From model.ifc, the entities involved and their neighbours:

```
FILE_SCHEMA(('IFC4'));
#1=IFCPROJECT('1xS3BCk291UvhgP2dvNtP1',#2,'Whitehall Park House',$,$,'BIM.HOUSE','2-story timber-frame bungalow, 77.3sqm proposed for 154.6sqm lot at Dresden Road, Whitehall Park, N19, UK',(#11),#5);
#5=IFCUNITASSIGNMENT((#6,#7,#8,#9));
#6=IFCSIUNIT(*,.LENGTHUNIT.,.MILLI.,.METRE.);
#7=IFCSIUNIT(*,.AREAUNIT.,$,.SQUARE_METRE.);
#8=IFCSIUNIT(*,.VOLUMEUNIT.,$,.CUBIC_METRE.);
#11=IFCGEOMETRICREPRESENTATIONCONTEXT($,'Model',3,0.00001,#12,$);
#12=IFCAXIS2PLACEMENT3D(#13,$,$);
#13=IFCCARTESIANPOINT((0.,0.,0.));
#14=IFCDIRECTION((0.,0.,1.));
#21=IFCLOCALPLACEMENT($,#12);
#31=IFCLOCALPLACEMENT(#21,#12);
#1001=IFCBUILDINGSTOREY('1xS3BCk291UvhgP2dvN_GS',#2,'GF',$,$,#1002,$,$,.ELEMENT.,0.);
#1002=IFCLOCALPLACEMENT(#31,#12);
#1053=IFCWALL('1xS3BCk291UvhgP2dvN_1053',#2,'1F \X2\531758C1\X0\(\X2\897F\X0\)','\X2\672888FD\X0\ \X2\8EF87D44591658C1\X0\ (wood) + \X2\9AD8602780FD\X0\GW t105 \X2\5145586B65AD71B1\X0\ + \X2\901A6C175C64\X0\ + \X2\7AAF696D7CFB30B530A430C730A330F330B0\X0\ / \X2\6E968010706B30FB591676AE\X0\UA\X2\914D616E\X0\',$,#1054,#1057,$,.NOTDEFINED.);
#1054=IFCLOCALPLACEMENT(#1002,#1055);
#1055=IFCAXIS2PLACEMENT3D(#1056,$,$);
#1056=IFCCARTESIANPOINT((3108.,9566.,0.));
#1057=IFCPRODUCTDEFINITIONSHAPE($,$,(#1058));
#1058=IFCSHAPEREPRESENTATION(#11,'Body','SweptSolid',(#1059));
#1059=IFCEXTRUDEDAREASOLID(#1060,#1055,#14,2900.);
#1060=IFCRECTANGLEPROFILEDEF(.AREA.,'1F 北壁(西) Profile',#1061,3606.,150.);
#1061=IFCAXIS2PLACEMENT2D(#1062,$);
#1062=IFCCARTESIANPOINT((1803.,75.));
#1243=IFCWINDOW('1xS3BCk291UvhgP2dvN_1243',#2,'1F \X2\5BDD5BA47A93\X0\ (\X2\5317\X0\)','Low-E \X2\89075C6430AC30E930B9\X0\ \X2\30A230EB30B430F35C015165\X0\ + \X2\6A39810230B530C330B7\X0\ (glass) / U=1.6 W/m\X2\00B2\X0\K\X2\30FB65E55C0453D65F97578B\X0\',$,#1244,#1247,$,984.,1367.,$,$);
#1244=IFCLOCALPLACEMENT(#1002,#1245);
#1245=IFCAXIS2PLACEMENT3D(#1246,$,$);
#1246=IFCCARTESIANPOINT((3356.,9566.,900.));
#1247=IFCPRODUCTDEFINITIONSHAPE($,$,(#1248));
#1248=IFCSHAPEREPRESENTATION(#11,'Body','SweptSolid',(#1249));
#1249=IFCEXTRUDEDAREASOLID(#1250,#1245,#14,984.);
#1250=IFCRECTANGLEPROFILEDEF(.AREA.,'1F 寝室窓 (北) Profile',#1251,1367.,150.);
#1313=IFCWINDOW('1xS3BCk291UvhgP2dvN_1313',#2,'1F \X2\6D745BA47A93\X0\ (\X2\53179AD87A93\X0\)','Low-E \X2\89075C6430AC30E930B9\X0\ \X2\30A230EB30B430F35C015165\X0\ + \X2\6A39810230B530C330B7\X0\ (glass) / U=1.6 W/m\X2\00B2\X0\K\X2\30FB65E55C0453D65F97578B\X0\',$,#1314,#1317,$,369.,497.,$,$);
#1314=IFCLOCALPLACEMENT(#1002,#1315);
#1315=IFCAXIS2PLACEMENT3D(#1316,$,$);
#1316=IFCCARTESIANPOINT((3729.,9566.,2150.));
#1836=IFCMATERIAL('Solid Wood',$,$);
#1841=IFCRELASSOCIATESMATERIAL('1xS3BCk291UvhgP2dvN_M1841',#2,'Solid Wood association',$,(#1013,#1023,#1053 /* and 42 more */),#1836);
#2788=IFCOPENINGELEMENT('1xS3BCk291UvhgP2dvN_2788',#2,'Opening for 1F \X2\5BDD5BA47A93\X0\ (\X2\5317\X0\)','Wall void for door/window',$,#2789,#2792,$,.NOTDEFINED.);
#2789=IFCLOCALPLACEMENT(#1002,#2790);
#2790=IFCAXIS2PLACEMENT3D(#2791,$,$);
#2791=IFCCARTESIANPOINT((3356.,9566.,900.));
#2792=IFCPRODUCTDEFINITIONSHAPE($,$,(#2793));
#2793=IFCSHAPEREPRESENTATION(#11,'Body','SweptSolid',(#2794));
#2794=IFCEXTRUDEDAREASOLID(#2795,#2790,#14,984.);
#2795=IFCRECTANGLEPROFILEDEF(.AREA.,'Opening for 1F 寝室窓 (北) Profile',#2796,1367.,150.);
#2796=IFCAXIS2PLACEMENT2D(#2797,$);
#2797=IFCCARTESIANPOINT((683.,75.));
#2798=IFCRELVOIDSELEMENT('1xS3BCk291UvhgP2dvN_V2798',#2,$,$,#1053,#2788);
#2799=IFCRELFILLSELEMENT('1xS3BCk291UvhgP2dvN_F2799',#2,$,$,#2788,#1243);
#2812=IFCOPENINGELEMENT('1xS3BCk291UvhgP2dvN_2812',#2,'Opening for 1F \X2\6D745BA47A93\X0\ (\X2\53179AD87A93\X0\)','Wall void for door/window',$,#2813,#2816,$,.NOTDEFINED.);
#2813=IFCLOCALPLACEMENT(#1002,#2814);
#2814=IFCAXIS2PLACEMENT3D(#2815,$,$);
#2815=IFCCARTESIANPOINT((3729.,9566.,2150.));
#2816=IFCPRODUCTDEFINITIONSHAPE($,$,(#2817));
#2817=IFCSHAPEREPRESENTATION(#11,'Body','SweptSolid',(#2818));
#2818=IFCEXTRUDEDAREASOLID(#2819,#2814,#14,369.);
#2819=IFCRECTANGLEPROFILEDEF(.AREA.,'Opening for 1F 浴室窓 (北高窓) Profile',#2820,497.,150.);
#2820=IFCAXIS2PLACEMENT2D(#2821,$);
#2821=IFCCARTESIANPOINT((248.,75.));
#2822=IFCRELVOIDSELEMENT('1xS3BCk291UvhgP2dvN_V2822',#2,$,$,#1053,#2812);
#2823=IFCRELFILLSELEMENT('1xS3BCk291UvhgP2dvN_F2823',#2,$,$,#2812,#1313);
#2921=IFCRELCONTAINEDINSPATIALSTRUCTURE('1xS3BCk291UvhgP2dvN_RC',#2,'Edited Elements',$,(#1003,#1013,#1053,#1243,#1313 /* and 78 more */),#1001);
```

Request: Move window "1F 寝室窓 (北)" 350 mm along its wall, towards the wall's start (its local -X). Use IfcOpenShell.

```python
import ifcopenshell
import ifcopenshell.api.geometry
import ifcopenshell.util.placement

model = ifcopenshell.open("model.ifc")

window = model.by_guid("1xS3BCk291UvhgP2dvN_1243")
opening = window.FillsVoids[0].RelatingOpeningElement
wall = opening.VoidsElements[0].RelatingBuildingElement

wall_matrix = ifcopenshell.util.placement.get_local_placement(wall.ObjectPlacement)
shift = wall_matrix[:3, 0] * -350.0
before = ifcopenshell.util.placement.get_local_placement(window.ObjectPlacement)[:3, 3].copy()

# The window is not placed relative to its opening, so move both.
for product in (opening, window):
    matrix = ifcopenshell.util.placement.get_local_placement(product.ObjectPlacement)
    matrix[:3, 3] += shift
    ifcopenshell.api.geometry.edit_object_placement(model, product=product, matrix=matrix, is_si=False)

after = ifcopenshell.util.placement.get_local_placement(window.ObjectPlacement)[:3, 3]
print("window moved by", (after - before).round(3) + 0.0)

model.write("model_edited.ifc")
```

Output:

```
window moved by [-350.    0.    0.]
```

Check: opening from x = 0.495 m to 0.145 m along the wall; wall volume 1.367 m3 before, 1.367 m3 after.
